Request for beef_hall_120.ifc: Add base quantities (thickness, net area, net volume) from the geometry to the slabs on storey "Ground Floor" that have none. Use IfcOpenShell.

First a look at what the model holds.

```python
import ifcopenshell
import ifcopenshell.util.element
import ifcopenshell.util.unit

model = ifcopenshell.open("beef_hall_120.ifc")
print(model.schema)
for unit_type in ("LENGTHUNIT", "AREAUNIT", "VOLUMEUNIT"):
    print(unit_type, ifcopenshell.util.unit.calculate_unit_scale(model, unit_type))
storey = next(s for s in model.by_type("IfcBuildingStorey") if s.Name == "Ground Floor")
slabs = [e for e in ifcopenshell.util.element.get_decomposition(storey) if e.is_a("IfcSlab")]
for e in sorted(slabs, key=lambda e: e.id()):
    print(e.id(), e.is_a(), e.Name, list(ifcopenshell.util.element.get_psets(e, qtos_only=True)), sep=" | ")
```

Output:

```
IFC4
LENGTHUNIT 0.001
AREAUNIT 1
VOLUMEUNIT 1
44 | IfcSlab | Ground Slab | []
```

```python
import ifcopenshell
import ifcopenshell.api.pset
import ifcopenshell.geom
import ifcopenshell.util.element
import ifcopenshell.util.shape
import ifcopenshell.util.unit

model = ifcopenshell.open("beef_hall_120.ifc")
unit_scale = ifcopenshell.util.unit.calculate_unit_scale(model)
area_scale = ifcopenshell.util.unit.calculate_unit_scale(model, "AREAUNIT")
volume_scale = ifcopenshell.util.unit.calculate_unit_scale(model, "VOLUMEUNIT")
settings = ifcopenshell.geom.settings()

storey = next(s for s in model.by_type("IfcBuildingStorey") if s.Name == "Ground Floor")
slabs = [e for e in ifcopenshell.util.element.get_decomposition(storey) if e.is_a("IfcSlab")]

for e in sorted(slabs, key=lambda e: e.id()):
    if ifcopenshell.util.element.get_psets(e, qtos_only=True, should_inherit=False):
        continue
    # Geometry comes back in metres, in the element's own axes.
    shape = ifcopenshell.geom.create_shape(settings, e)
    values = {
        "Width": ifcopenshell.util.shape.get_z(shape.geometry) / unit_scale,
        "NetArea": ifcopenshell.util.shape.get_footprint_area(shape.geometry) / area_scale,
        "NetVolume": ifcopenshell.util.shape.get_volume(shape.geometry) / volume_scale,
    }
    qto = ifcopenshell.api.pset.add_qto(model, product=e, name="Qto_SlabBaseQuantities")
    ifcopenshell.api.pset.edit_qto(model, qto=qto, properties=values)
    print(e.id(), {k: round(v, 3) for k, v in values.items()})

model.write("beef_hall_120_v2.ifc")
```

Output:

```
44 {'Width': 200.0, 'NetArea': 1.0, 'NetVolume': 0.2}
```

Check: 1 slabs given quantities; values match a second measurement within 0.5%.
